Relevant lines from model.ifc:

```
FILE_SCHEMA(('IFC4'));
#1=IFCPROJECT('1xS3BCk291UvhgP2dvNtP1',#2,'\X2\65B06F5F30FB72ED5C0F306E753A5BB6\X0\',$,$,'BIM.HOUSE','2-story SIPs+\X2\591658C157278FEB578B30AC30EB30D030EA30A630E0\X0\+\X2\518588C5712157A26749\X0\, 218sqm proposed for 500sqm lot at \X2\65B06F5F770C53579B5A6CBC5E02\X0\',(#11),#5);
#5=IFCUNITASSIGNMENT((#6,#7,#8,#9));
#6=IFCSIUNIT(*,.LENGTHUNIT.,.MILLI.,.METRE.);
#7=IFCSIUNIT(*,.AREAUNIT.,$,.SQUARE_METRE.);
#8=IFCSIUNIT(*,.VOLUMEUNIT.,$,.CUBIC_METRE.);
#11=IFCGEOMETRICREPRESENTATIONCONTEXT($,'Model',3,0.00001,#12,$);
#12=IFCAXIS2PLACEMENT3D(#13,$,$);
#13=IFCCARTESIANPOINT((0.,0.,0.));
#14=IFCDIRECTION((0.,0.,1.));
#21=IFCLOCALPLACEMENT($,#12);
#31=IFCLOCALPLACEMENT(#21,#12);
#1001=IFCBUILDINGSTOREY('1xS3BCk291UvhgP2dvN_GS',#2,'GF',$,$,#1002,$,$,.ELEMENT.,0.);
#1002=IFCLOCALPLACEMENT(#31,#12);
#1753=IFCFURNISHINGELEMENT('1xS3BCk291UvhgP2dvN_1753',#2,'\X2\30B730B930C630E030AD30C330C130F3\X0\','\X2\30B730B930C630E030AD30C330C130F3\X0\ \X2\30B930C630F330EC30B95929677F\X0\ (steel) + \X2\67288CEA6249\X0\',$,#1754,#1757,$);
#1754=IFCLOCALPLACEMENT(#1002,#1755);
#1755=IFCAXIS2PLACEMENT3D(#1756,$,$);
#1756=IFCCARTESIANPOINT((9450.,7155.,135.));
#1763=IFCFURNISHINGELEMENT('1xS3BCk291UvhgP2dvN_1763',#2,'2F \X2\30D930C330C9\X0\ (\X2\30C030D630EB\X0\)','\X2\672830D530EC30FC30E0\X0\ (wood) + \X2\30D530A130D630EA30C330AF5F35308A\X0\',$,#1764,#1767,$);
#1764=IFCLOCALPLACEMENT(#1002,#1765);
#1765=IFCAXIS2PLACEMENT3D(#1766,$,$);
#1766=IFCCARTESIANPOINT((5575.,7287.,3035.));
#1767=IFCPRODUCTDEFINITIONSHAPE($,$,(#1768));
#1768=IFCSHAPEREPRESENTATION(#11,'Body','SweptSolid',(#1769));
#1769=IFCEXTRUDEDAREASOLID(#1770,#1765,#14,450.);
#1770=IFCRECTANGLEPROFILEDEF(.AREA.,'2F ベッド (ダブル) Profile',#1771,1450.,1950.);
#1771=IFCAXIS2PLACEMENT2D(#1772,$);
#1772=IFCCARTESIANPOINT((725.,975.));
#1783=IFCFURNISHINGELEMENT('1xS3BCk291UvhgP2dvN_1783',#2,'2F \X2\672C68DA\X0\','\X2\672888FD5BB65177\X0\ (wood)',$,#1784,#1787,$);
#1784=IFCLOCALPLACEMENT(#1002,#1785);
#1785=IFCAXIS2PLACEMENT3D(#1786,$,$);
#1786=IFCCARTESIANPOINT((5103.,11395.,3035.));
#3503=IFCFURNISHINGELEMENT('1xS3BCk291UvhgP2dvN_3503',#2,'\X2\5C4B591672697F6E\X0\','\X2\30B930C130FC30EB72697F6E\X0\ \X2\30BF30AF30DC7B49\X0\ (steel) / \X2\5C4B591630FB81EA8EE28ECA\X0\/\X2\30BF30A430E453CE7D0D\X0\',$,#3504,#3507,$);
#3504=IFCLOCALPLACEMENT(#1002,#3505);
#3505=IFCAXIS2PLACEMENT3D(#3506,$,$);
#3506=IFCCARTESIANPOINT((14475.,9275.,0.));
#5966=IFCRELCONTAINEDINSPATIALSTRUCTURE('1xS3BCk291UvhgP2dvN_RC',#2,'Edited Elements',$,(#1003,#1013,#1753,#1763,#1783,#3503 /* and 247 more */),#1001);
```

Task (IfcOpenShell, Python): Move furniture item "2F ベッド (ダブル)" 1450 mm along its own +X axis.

```python
import ifcopenshell
import ifcopenshell.api.geometry
import ifcopenshell.util.placement
import ifcopenshell.util.unit

model = ifcopenshell.open("model.ifc")
unit_scale = ifcopenshell.util.unit.calculate_unit_scale(model)

item = model.by_guid("1xS3BCk291UvhgP2dvN_1763")
matrix = ifcopenshell.util.placement.get_local_placement(item.ObjectPlacement)
matrix[:3, 3] += matrix[:3, 0] * 1.45 / unit_scale
ifcopenshell.api.geometry.edit_object_placement(model, product=item, matrix=matrix, is_si=False)

print(ifcopenshell.util.placement.get_local_placement(item.ObjectPlacement).round(3) + 0.0)

model.write("model_edited.ifc")
```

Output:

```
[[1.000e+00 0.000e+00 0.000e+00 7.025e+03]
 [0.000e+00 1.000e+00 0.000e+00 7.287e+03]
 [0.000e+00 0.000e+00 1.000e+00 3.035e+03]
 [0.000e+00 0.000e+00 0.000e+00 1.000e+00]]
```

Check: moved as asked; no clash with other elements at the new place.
